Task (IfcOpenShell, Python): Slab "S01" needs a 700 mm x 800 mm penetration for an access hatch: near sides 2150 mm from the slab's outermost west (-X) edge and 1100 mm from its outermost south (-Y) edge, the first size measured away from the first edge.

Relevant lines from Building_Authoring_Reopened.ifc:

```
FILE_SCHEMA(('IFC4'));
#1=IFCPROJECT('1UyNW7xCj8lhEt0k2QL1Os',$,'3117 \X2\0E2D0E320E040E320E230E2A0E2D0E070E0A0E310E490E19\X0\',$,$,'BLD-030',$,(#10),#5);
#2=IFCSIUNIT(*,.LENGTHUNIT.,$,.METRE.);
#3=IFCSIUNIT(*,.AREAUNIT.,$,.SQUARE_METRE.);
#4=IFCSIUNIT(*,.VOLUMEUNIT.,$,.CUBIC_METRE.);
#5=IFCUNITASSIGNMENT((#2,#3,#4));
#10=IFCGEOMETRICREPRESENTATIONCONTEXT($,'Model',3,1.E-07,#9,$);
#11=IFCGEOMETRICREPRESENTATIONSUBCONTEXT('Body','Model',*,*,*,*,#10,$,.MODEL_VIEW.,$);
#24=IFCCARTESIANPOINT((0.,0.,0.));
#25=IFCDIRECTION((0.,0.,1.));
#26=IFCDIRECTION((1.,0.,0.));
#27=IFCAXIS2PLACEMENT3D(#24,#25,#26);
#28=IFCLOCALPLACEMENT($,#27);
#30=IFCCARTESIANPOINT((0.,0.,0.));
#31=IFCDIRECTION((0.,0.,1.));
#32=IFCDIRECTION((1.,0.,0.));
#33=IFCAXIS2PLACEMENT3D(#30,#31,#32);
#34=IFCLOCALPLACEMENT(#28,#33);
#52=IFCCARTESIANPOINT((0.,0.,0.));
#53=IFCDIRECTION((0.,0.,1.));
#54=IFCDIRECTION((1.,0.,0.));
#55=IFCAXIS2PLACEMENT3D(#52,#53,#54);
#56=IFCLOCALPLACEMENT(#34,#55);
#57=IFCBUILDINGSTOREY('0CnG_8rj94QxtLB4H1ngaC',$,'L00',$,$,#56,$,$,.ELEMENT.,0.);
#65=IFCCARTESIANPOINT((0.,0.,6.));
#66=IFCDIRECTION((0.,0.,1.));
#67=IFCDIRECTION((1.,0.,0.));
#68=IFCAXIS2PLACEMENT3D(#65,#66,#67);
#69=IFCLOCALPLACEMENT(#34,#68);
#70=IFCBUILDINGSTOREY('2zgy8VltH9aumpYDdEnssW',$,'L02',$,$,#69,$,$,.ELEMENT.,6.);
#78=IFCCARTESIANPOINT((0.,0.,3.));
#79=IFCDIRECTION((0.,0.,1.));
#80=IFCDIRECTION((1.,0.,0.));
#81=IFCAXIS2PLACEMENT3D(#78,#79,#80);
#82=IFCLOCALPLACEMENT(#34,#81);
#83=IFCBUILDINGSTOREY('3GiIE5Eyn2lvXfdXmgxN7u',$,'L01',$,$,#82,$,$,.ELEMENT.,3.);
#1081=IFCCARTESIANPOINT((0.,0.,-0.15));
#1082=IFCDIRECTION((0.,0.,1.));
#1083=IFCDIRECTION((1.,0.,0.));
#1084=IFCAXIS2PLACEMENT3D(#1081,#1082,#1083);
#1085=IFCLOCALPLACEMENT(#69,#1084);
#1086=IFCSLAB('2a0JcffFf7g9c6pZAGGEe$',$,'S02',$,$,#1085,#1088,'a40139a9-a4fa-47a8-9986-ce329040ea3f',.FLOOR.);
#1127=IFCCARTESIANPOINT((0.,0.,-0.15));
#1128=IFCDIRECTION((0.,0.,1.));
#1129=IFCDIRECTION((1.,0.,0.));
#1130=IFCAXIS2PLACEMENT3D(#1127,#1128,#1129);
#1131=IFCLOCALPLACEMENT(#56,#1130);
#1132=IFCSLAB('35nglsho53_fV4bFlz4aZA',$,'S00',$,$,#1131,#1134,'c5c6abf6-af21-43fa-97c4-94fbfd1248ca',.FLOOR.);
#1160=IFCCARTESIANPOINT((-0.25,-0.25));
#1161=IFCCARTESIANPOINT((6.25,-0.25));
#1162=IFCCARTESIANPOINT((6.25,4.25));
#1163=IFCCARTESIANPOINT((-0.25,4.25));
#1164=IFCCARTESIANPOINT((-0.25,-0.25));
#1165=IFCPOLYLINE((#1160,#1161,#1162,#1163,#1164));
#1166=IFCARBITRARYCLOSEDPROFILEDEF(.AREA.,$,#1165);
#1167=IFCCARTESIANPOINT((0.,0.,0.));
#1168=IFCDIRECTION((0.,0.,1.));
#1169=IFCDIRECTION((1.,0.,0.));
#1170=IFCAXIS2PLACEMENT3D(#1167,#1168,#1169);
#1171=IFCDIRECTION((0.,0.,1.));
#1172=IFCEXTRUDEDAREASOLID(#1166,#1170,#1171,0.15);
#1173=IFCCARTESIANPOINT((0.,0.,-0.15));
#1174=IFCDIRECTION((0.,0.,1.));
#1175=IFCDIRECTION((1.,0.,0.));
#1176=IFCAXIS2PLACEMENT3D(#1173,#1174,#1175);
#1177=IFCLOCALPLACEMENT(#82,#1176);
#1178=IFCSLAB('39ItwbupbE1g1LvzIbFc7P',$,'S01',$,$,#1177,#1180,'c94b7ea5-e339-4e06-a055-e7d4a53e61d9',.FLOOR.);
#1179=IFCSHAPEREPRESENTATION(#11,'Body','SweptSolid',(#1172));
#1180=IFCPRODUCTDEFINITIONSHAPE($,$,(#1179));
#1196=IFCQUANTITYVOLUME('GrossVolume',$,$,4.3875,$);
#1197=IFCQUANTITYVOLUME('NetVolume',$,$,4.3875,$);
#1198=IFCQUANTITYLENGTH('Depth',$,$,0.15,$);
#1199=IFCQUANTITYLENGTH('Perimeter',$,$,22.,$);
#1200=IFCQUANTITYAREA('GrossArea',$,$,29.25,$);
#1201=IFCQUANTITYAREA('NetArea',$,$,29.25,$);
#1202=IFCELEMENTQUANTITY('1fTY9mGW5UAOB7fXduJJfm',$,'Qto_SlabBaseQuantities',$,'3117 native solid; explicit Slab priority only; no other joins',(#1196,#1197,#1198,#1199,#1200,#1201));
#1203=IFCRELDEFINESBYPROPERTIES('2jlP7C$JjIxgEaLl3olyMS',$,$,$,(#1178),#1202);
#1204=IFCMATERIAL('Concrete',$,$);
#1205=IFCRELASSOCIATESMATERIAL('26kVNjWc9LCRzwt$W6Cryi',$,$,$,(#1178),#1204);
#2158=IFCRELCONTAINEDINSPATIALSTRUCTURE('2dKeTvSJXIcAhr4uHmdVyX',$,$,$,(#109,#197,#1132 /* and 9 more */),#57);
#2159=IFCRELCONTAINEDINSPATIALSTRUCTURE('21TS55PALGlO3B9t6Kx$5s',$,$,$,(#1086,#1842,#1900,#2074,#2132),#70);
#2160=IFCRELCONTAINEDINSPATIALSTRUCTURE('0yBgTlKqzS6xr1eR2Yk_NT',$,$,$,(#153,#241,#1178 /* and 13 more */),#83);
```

```python
import numpy as np
import ifcopenshell
import ifcopenshell.api.feature
import ifcopenshell.api.geometry
import ifcopenshell.api.pset
import ifcopenshell.api.root
import ifcopenshell.geom
import ifcopenshell.util.element
import ifcopenshell.util.placement
import ifcopenshell.util.representation
import ifcopenshell.util.shape
import ifcopenshell.util.unit

model = ifcopenshell.open("Building_Authoring_Reopened.ifc")
unit_scale = ifcopenshell.util.unit.calculate_unit_scale(model)
area_scale = ifcopenshell.util.unit.calculate_unit_scale(model, "AREAUNIT")
volume_scale = ifcopenshell.util.unit.calculate_unit_scale(model, "VOLUMEUNIT")
settings = ifcopenshell.geom.settings()


def volume(element):
    """Net volume in cubic metres, openings subtracted."""
    shape = ifcopenshell.geom.create_shape(settings, element)
    return ifcopenshell.util.shape.get_volume(shape.geometry)


slab = model.by_id(1178)
before = volume(slab)

# Extent in the slab's own axes, in metres. The edges named are its -X and -Y sides.
slab_shape = ifcopenshell.geom.create_shape(settings, slab)
vertices = ifcopenshell.util.shape.get_vertices(slab_shape.geometry)
x_min, y_min, bottom = vertices.min(axis=0)
top = vertices[:, 2].max()

opening = ifcopenshell.api.root.create_entity(model, ifc_class="IfcOpeningElement", name="Access hatch opening", predefined_type="OPENING")
context = ifcopenshell.util.representation.get_context(model, "Model", "Body", "MODEL_VIEW")
width, depth = 0.7, 0.8
outline = [(0.0, 0.0), (width, 0.0), (width, depth), (0.0, depth), (0.0, 0.0)]
# Overshoot both faces by 50 mm so the cut is clean.
shape = ifcopenshell.api.geometry.add_slab_representation(
    model, context=context, depth=top - bottom + 0.1, polyline=outline
)
ifcopenshell.api.geometry.assign_representation(model, product=opening, representation=shape)

matrix = ifcopenshell.util.placement.get_local_placement(slab.ObjectPlacement)
matrix[:, 3] = matrix @ np.append(np.array([x_min + 2.15, y_min + 1.1, bottom - 0.05]) / unit_scale, 1.0)
ifcopenshell.api.geometry.edit_object_placement(model, product=opening, matrix=matrix, is_si=False)
ifcopenshell.api.feature.add_feature(model, feature=opening, element=slab)

after = volume(slab)

# Update the slab's stored quantities.
qto = model.by_id(ifcopenshell.util.element.get_pset(slab, "Qto_SlabBaseQuantities", should_inherit=False)["id"])
ifcopenshell.api.pset.edit_qto(model, qto=qto, properties={
    "NetVolume": after / volume_scale,
    "NetArea": after / (top - bottom) / area_scale,
})

print(f"slab volume {before:.3f} -> {after:.3f} m3")

model.write("Building_Authoring_Reopened_updated.ifc")
```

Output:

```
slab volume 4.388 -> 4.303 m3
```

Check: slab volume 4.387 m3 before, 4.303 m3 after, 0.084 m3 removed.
